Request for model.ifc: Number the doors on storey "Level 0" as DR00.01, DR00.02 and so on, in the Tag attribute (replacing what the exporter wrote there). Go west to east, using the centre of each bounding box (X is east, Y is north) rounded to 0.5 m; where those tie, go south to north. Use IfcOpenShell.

First a look at what the model holds.

```python
import ifcopenshell
import ifcopenshell.util.element
import ifcopenshell.util.placement

model = ifcopenshell.open("model.ifc")
print(model.schema)
storey = next(s for s in model.by_type("IfcBuildingStorey") if s.Name == "Level 0")
doors = [e for e in ifcopenshell.util.element.get_decomposition(storey) if e.is_a("IfcDoor")]
for e in sorted(doors, key=lambda e: e.id()):
    origin = ifcopenshell.util.placement.get_local_placement(e.ObjectPlacement)[:3, 3]
    print(e.id(), e.Tag, e.Name, origin.round(2) + 0.0, sep=" | ")
```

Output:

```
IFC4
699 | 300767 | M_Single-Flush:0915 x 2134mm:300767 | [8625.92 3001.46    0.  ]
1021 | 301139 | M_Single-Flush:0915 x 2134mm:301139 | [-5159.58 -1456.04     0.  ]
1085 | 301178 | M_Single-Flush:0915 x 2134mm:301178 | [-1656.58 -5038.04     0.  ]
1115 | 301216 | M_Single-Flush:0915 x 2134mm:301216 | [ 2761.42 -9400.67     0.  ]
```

```python
import ifcopenshell
import ifcopenshell.geom
import ifcopenshell.util.element
import ifcopenshell.util.shape

model = ifcopenshell.open("model.ifc")
settings = ifcopenshell.geom.settings()
settings.set("use-world-coords", True)


def centre(element):
    shape = ifcopenshell.geom.create_shape(settings, element)
    return ifcopenshell.util.shape.get_bbox_centroid(shape.geometry)


storey = next(s for s in model.by_type("IfcBuildingStorey") if s.Name == "Level 0")
doors = [e for e in ifcopenshell.util.element.get_decomposition(storey) if e.is_a("IfcDoor")]

# Insertion points can sit at a corner or the storey origin, so sort by the geometry (in metres).
centres = {e: centre(e) for e in doors}
doors.sort(key=lambda e: (round(centres[e][0] / 0.5), centres[e][1]))

for i, e in enumerate(doors, start=1):
    number = f"DR00.{i:02d}"
    e.Tag = number
    print(e.id(), number)

model.write("model_rev.ifc")
```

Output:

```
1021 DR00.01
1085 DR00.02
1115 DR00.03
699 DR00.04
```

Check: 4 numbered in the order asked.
